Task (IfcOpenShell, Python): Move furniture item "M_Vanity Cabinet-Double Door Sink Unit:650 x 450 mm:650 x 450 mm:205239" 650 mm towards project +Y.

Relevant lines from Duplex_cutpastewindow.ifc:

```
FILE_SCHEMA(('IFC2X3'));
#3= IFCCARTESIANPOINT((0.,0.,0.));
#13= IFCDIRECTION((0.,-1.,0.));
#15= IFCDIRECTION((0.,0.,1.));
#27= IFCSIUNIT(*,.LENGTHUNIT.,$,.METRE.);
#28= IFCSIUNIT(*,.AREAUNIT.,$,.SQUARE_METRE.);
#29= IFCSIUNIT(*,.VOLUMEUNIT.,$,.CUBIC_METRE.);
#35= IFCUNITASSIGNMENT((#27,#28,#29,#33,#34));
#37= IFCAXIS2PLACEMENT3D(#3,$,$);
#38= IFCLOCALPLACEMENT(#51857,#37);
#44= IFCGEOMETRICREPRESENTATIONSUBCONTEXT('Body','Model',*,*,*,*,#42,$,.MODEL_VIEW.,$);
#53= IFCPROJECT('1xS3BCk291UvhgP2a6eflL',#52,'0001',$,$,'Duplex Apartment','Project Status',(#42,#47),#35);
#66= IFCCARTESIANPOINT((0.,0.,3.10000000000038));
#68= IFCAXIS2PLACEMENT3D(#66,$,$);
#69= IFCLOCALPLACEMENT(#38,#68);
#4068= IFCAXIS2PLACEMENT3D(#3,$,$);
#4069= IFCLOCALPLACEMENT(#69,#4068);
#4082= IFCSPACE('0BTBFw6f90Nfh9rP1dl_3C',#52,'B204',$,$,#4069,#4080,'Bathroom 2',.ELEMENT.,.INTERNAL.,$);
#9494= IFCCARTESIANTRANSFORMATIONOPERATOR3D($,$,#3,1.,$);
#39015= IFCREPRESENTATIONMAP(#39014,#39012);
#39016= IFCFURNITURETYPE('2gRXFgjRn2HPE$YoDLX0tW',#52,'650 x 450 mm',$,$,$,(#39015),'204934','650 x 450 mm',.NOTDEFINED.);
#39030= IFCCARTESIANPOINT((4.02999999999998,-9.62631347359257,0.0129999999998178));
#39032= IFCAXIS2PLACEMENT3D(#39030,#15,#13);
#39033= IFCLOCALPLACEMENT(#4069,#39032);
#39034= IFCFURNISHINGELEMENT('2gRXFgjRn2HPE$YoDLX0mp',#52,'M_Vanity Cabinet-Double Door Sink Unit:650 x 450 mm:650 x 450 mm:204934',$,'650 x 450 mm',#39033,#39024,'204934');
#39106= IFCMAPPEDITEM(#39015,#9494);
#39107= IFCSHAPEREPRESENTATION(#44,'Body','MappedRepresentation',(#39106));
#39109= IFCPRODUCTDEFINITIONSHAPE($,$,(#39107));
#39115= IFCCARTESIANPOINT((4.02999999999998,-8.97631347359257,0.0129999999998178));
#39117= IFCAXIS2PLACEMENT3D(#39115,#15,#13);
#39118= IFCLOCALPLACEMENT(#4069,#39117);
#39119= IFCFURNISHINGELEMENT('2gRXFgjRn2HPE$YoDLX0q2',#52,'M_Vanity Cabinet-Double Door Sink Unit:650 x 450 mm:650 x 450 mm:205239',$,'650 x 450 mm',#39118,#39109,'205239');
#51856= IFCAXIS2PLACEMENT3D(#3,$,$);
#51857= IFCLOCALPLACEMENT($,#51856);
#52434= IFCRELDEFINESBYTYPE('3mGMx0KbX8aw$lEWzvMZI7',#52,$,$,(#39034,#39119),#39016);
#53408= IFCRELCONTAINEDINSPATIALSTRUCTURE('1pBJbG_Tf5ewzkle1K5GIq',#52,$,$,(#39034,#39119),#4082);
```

```python
import ifcopenshell
import ifcopenshell.api.geometry
import ifcopenshell.util.placement
import ifcopenshell.util.unit

model = ifcopenshell.open("Duplex_cutpastewindow.ifc")
unit_scale = ifcopenshell.util.unit.calculate_unit_scale(model)

item = model.by_guid("2gRXFgjRn2HPE$YoDLX0q2")
matrix = ifcopenshell.util.placement.get_local_placement(item.ObjectPlacement)
matrix[1, 3] += 0.65 / unit_scale
ifcopenshell.api.geometry.edit_object_placement(model, product=item, matrix=matrix, is_si=False)

print(ifcopenshell.util.placement.get_local_placement(item.ObjectPlacement).round(3) + 0.0)

model.write("Duplex_cutpastewindow_edited.ifc")
```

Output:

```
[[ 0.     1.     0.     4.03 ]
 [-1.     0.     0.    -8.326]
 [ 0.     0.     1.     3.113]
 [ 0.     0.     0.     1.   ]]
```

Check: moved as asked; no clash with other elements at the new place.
